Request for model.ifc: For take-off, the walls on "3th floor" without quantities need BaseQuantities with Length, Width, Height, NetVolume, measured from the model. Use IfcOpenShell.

First a look at what the model holds.

```python
import ifcopenshell
import ifcopenshell.util.element
import ifcopenshell.util.unit

model = ifcopenshell.open("model.ifc")
print(model.schema)
for unit_type in ("LENGTHUNIT", "AREAUNIT", "VOLUMEUNIT"):
    print(unit_type, ifcopenshell.util.unit.calculate_unit_scale(model, unit_type))
storey = next(s for s in model.by_type("IfcBuildingStorey") if s.Name == "3th floor")
walls = [e for e in ifcopenshell.util.element.get_decomposition(storey) if e.is_a("IfcWall")]
for e in sorted(walls, key=lambda e: e.id()):
    print(e.id(), e.is_a(), e.Name, list(ifcopenshell.util.element.get_psets(e, qtos_only=True)), sep=" | ")
```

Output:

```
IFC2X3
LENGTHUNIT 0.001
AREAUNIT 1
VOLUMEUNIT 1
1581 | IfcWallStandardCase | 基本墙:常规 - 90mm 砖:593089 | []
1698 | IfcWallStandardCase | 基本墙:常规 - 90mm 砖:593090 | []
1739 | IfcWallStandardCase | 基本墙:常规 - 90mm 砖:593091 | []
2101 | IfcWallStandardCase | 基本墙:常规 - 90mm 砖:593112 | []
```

```python
import ifcopenshell
import ifcopenshell.api.pset
import ifcopenshell.geom
import ifcopenshell.util.element
import ifcopenshell.util.shape
import ifcopenshell.util.unit

model = ifcopenshell.open("model.ifc")
unit_scale = ifcopenshell.util.unit.calculate_unit_scale(model)
volume_scale = ifcopenshell.util.unit.calculate_unit_scale(model, "VOLUMEUNIT")
settings = ifcopenshell.geom.settings()

storey = next(s for s in model.by_type("IfcBuildingStorey") if s.Name == "3th floor")
walls = [e for e in ifcopenshell.util.element.get_decomposition(storey) if e.is_a("IfcWall")]

for e in sorted(walls, key=lambda e: e.id()):
    if ifcopenshell.util.element.get_psets(e, qtos_only=True, should_inherit=False):
        continue
    # Geometry comes back in metres, in the element's own axes.
    shape = ifcopenshell.geom.create_shape(settings, e)
    values = {
        "Length": ifcopenshell.util.shape.get_x(shape.geometry) / unit_scale,
        "Width": ifcopenshell.util.shape.get_y(shape.geometry) / unit_scale,
        "Height": ifcopenshell.util.shape.get_z(shape.geometry) / unit_scale,
        "NetVolume": ifcopenshell.util.shape.get_volume(shape.geometry) / volume_scale,
    }
    qto = ifcopenshell.api.pset.add_qto(model, product=e, name="BaseQuantities")
    ifcopenshell.api.pset.edit_qto(model, qto=qto, properties=values)
    print(e.id(), {k: round(v, 3) for k, v in values.items()})

model.write("model-out.ifc")
```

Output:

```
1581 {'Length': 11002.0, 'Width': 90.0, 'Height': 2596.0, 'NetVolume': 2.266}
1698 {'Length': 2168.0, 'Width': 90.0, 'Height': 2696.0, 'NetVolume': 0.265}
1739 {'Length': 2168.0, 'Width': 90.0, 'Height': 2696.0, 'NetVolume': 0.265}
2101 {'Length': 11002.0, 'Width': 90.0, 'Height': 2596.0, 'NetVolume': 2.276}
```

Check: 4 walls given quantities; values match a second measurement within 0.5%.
